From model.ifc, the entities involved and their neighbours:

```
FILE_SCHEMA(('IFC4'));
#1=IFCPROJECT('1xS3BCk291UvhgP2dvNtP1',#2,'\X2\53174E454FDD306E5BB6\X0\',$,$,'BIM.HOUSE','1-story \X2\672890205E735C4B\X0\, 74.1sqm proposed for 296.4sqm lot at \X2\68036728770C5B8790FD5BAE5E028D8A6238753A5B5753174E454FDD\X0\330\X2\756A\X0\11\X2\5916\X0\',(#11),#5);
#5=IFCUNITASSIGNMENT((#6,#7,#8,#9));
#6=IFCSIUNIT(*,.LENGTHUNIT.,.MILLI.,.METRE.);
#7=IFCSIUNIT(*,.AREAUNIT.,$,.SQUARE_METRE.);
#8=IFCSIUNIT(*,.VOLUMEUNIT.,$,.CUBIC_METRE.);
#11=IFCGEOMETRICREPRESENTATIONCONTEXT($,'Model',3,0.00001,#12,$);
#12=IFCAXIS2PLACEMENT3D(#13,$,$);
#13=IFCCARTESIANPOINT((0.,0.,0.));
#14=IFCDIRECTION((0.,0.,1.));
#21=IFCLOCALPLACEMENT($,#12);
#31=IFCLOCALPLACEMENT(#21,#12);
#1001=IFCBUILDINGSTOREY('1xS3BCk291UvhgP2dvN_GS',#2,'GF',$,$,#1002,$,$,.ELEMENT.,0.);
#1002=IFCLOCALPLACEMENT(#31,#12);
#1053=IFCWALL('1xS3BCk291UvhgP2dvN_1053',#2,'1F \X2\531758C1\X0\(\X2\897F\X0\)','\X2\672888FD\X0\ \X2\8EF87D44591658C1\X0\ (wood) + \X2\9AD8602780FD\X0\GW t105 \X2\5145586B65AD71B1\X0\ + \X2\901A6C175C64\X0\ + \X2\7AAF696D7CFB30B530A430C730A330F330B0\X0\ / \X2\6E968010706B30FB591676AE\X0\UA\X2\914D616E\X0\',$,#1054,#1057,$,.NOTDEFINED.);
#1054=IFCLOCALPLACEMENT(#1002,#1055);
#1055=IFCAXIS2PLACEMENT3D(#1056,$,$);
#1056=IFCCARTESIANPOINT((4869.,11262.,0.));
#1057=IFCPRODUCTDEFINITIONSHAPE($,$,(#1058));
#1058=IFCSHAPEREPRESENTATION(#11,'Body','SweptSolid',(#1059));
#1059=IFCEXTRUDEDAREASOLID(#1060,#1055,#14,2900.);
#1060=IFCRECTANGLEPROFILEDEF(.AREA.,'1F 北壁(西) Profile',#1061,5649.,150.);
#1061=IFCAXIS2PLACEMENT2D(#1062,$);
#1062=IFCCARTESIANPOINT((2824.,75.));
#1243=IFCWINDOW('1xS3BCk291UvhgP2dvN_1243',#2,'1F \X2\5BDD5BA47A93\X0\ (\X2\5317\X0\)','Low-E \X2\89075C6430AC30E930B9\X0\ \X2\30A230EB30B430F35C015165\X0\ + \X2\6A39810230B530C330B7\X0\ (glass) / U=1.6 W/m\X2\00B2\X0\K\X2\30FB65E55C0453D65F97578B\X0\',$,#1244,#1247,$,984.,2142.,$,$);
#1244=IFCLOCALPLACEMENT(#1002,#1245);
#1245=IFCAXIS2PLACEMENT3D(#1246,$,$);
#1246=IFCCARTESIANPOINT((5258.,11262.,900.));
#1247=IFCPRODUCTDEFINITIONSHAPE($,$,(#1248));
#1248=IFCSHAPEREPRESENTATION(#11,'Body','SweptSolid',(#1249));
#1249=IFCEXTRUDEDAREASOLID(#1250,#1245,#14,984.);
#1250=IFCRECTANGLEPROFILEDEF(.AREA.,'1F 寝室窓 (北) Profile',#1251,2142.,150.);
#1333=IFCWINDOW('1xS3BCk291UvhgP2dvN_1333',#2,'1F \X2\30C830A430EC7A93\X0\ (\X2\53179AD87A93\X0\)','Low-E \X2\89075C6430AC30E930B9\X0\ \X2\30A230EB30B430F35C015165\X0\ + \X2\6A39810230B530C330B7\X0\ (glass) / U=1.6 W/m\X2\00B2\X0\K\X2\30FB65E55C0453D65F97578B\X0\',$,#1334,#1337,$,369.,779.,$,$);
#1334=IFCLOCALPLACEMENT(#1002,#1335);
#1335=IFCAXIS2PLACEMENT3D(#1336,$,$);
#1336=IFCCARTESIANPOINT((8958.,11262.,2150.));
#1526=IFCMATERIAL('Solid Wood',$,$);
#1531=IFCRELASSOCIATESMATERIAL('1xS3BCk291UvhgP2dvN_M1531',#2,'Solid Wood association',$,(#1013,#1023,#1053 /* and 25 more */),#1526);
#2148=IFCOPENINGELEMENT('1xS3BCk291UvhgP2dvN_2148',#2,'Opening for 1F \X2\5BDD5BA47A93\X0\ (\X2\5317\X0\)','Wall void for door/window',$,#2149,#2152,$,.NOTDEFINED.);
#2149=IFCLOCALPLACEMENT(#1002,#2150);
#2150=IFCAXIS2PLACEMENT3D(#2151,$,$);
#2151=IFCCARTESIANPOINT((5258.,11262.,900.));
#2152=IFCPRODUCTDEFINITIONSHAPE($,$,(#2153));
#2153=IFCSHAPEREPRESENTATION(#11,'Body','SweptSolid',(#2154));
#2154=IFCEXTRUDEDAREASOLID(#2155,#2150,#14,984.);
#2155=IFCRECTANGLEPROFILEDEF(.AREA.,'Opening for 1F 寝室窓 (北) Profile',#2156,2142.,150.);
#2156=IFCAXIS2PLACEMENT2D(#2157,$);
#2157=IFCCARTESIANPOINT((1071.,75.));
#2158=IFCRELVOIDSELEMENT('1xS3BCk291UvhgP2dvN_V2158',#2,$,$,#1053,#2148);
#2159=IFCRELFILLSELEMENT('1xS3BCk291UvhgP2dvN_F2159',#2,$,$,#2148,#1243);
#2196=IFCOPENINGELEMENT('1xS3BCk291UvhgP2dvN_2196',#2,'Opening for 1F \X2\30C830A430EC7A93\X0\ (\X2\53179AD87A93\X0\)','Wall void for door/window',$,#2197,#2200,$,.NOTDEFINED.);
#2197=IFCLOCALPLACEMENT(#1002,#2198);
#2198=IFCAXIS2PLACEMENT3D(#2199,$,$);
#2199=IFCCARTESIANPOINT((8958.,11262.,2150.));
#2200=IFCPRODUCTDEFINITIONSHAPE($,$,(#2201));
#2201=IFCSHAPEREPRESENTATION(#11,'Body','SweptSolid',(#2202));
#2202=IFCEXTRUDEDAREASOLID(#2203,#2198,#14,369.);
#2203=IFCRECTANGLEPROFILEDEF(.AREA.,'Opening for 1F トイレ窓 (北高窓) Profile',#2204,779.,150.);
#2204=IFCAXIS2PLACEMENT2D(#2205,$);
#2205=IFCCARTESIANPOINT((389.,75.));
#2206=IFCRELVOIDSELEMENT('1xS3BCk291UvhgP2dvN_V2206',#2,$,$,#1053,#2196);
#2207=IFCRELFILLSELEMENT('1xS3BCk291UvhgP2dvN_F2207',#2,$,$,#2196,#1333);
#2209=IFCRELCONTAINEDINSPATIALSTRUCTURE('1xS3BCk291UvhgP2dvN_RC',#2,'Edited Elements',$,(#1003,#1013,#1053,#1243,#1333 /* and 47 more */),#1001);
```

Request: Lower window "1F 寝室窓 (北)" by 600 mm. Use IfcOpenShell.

```python
import numpy as np
import ifcopenshell
import ifcopenshell.api.geometry
import ifcopenshell.util.placement
import ifcopenshell.util.unit

model = ifcopenshell.open("model.ifc")
unit_scale = ifcopenshell.util.unit.calculate_unit_scale(model)

window = model.by_guid("1xS3BCk291UvhgP2dvN_1243")
opening = window.FillsVoids[0].RelatingOpeningElement
dz = -0.6 / unit_scale

shift = np.array([0.0, 0.0, dz])
# The window is not placed relative to its opening, so move both.
for product in (opening, window):
    matrix = ifcopenshell.util.placement.get_local_placement(product.ObjectPlacement)
    matrix[:3, 3] += shift
    ifcopenshell.api.geometry.edit_object_placement(model, product=product, matrix=matrix, is_si=False)

print(f"moved by {dz * unit_scale:+.3f} m")

model.write("model-out.ifc")
```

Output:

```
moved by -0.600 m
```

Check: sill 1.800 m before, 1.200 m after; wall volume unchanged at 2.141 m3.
